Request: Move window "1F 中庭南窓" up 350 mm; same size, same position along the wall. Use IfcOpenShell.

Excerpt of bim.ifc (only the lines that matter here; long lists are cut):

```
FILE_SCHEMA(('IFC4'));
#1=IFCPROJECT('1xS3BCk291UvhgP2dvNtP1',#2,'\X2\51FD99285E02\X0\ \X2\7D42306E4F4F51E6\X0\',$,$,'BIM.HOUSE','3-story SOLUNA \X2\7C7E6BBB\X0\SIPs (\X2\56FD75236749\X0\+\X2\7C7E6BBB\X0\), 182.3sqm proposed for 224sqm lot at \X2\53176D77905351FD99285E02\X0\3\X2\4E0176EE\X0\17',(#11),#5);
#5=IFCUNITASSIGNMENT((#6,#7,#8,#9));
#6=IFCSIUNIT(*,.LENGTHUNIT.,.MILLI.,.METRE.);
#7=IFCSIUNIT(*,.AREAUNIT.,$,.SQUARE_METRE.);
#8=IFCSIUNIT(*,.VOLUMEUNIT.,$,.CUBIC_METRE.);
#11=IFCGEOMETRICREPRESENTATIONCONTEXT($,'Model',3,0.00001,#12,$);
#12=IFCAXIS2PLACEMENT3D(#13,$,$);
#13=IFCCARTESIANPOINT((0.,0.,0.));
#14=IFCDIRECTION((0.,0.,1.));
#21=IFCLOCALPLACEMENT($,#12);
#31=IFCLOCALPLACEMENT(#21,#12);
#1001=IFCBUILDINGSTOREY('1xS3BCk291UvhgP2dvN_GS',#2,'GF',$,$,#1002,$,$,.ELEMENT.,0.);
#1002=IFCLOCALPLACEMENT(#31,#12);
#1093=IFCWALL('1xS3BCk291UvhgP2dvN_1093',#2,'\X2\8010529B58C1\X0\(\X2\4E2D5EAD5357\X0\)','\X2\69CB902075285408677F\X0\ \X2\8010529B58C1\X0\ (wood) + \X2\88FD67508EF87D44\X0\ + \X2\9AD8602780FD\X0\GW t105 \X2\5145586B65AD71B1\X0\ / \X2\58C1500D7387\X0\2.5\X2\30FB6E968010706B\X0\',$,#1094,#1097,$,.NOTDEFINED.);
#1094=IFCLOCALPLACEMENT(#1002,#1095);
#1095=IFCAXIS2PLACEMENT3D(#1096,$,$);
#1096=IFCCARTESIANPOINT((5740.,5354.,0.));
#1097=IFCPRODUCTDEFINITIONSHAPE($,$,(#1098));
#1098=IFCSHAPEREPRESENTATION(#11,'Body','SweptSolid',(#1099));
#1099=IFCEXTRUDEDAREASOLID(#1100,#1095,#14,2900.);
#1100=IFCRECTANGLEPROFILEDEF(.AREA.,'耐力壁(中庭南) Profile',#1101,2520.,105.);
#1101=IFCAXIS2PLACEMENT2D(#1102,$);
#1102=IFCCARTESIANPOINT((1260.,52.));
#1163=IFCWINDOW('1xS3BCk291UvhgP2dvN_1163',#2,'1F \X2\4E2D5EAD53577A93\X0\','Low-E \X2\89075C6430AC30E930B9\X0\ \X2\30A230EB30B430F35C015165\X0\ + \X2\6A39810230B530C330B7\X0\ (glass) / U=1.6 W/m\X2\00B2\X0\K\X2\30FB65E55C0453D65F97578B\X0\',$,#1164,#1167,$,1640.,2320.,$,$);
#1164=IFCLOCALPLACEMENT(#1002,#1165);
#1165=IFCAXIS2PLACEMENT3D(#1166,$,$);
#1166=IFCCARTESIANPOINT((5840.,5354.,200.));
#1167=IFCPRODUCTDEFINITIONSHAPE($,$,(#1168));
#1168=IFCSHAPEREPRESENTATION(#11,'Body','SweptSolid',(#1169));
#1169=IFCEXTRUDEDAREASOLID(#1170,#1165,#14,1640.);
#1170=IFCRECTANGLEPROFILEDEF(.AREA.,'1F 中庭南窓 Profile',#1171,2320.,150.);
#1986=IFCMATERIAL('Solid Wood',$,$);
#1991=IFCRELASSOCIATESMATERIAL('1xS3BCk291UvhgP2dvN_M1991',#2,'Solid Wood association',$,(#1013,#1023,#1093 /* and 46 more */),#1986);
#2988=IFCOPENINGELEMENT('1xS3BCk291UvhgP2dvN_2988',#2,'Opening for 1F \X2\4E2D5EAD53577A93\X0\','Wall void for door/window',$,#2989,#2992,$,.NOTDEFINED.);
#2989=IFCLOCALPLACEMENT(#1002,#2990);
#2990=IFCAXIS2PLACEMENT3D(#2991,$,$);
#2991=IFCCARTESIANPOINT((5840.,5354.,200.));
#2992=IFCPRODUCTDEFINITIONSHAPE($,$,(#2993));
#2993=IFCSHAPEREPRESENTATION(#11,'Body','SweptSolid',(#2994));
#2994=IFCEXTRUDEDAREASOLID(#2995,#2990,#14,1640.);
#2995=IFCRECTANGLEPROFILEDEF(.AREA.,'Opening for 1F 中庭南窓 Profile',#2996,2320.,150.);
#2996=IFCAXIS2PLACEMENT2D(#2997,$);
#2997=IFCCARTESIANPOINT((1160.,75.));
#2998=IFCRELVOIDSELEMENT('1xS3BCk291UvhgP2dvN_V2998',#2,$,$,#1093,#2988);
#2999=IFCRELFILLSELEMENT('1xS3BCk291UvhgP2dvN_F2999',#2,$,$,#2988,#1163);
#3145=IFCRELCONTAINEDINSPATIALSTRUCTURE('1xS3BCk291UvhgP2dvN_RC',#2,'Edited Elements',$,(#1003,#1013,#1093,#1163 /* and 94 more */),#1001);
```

```python
import numpy as np
import ifcopenshell
import ifcopenshell.api.geometry
import ifcopenshell.util.placement
import ifcopenshell.util.unit

model = ifcopenshell.open("bim.ifc")
unit_scale = ifcopenshell.util.unit.calculate_unit_scale(model)

window = model.by_guid("1xS3BCk291UvhgP2dvN_1163")
opening = window.FillsVoids[0].RelatingOpeningElement
dz = 0.35 / unit_scale

shift = np.array([0.0, 0.0, dz])
# The window is not placed relative to its opening, so move both.
for product in (opening, window):
    matrix = ifcopenshell.util.placement.get_local_placement(product.ObjectPlacement)
    matrix[:3, 3] += shift
    ifcopenshell.api.geometry.edit_object_placement(model, product=product, matrix=matrix, is_si=False)

print(f"moved by {dz * unit_scale:+.3f} m")

model.write("bim_updated.ifc")
```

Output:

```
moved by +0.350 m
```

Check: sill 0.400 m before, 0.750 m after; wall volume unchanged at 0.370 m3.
